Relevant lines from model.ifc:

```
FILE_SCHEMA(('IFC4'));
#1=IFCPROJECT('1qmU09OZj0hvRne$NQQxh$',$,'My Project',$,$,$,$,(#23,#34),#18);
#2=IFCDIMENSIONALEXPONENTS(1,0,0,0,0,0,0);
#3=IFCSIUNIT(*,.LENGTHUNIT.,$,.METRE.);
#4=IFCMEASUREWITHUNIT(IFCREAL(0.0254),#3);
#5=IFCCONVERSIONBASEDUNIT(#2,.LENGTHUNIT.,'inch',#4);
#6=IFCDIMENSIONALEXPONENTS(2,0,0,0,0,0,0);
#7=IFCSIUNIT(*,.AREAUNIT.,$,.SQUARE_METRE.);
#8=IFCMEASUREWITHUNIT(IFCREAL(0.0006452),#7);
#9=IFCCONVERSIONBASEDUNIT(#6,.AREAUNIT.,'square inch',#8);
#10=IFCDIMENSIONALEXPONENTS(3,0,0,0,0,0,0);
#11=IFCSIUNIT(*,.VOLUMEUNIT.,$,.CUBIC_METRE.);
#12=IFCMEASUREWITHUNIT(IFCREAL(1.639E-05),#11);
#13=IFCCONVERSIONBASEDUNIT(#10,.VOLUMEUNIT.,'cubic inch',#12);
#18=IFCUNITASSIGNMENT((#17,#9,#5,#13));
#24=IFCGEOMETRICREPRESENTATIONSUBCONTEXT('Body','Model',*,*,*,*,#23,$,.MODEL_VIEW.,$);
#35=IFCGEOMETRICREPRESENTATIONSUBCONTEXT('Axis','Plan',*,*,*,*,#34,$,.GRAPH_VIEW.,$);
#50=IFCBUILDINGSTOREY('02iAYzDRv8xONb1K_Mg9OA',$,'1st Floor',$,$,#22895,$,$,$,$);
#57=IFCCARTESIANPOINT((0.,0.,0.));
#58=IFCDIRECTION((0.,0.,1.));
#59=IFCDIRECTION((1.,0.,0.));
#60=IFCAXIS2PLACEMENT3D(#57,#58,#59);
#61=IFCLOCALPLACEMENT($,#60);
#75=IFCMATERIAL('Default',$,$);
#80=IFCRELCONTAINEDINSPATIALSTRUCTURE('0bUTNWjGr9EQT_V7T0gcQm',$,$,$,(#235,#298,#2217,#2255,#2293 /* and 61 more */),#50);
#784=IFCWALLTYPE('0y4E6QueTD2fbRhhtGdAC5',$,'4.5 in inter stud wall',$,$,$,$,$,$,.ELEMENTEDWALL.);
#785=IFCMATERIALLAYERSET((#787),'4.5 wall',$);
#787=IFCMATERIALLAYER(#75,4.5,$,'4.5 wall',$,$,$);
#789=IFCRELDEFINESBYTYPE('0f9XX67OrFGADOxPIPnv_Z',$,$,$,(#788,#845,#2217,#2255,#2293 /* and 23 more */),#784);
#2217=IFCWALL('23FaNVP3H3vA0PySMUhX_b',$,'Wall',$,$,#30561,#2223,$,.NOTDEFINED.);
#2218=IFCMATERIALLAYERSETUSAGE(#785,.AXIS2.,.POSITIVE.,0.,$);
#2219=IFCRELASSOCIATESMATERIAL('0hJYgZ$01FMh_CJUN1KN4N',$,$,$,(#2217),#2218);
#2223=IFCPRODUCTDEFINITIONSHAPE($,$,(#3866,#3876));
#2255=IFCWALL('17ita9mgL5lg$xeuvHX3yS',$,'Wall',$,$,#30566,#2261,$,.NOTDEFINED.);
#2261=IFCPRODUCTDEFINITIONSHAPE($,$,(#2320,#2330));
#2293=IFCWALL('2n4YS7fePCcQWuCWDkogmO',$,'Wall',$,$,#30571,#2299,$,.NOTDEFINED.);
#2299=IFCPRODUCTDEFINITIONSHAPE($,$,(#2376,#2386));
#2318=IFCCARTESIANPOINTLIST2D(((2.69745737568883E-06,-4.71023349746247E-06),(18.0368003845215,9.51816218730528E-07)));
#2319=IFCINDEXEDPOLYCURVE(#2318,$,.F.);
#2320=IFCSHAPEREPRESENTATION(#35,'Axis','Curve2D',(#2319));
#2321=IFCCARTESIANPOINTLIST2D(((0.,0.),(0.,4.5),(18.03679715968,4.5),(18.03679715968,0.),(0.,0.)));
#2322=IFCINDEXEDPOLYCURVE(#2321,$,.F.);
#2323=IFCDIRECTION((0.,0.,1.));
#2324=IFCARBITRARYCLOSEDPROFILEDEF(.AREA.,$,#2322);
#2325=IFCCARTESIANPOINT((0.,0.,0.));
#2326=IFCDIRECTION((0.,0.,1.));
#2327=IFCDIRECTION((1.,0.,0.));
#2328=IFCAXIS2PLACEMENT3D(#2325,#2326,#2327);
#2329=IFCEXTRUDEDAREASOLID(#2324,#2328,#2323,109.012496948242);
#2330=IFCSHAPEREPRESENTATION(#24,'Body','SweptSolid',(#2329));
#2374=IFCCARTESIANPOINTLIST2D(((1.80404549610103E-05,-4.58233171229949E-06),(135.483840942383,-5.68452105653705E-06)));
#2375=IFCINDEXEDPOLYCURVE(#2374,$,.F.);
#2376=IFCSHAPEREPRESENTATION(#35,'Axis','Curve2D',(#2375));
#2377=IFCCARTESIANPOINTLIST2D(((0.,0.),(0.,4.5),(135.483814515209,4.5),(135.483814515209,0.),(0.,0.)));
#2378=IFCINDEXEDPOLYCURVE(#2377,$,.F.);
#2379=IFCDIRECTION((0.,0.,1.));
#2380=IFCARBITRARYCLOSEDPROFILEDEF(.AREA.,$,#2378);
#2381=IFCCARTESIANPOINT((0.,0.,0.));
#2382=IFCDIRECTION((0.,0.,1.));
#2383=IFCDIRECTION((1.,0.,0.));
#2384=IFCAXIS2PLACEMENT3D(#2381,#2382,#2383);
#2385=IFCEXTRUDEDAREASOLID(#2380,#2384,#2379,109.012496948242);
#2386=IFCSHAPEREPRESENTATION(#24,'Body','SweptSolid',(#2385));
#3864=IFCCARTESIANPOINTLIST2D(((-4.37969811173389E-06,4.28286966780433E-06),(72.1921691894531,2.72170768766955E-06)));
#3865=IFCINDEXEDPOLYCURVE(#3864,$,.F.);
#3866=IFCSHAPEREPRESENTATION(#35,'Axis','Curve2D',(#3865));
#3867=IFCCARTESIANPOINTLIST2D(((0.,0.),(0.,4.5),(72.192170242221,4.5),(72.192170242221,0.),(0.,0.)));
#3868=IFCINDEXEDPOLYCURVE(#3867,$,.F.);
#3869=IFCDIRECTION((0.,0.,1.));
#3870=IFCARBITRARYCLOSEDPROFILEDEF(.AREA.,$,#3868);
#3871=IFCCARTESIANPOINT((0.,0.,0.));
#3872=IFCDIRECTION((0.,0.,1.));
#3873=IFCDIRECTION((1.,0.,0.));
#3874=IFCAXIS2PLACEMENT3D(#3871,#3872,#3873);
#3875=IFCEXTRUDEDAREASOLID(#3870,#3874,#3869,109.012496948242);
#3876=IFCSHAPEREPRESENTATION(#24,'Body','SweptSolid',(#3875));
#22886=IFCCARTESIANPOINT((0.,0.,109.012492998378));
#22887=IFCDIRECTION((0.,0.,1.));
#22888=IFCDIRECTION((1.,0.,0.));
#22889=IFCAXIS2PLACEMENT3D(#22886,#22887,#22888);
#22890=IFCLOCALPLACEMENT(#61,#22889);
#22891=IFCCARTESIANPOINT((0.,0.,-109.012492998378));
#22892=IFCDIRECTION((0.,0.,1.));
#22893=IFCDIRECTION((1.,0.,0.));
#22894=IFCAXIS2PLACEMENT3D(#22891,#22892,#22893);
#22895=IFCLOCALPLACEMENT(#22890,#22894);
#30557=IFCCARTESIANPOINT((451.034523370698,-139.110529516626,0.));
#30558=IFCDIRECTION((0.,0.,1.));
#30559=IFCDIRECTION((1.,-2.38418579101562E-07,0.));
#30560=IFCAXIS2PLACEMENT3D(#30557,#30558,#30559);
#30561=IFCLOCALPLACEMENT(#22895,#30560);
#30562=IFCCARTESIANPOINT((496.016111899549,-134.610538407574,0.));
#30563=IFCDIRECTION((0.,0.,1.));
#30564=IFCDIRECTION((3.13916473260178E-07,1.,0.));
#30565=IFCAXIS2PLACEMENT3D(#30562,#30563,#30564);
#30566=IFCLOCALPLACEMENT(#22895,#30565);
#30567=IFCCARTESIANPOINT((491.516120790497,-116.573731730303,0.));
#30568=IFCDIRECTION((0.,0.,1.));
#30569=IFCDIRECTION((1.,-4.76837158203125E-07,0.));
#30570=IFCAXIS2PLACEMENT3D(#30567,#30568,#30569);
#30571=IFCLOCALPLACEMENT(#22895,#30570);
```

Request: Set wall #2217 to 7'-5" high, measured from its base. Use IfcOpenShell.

```python
import ifcopenshell
import ifcopenshell.geom
import ifcopenshell.util.representation
import ifcopenshell.util.shape
import ifcopenshell.util.unit

model = ifcopenshell.open("model.ifc")
unit_scale = ifcopenshell.util.unit.calculate_unit_scale(model)
settings = ifcopenshell.geom.settings()


def volume(element):
    """Net volume in cubic metres, openings subtracted."""
    shape = ifcopenshell.geom.create_shape(settings, element)
    return ifcopenshell.util.shape.get_volume(shape.geometry)


wall = model.by_id(2217)
before = volume(wall)

body = ifcopenshell.util.representation.get_representation(wall, "Model", "Body")
solid = body.Items[0]
old_height = solid.Depth
solid.Depth = 89 * 0.0254 / unit_scale
after = volume(wall)

print(f"height {old_height:g} -> {solid.Depth:g}, volume {before:.3f} -> {after:.3f} m3")

model.write("model_rev.ifc")
```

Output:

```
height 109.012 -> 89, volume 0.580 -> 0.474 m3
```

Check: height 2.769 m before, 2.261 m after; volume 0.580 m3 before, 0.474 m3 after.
